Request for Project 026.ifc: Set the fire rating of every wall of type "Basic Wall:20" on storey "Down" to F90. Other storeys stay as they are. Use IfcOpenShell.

First a look at what the model holds.

```python
import ifcopenshell
import ifcopenshell.util.element

model = ifcopenshell.open("Project 026.ifc")
print(model.schema)
storey = next(s for s in model.by_type("IfcBuildingStorey") if s.Name == "Down")
walls = [e for e in ifcopenshell.util.element.get_decomposition(storey) if e.is_a("IfcWall")]
seen = {}
for e in walls:
    element_type = ifcopenshell.util.element.get_type(e)
    key = (element_type.Name if element_type != e and element_type else None, ifcopenshell.util.element.get_pset(e, "Pset_WallCommon", "FireRating"))
    seen[key] = seen.get(key, 0) + 1
for (name, value), count in sorted(seen.items(), key=str):
    print(count, "x", name, "|", value)
```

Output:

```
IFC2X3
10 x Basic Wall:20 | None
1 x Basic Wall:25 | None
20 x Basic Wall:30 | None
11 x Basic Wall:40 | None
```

```python
import ifcopenshell
import ifcopenshell.api.pset
import ifcopenshell.util.element

model = ifcopenshell.open("Project 026.ifc")

storey = next(s for s in model.by_type("IfcBuildingStorey") if s.Name == "Down")
walls = [e for e in ifcopenshell.util.element.get_decomposition(storey) if e.is_a("IfcWall")]

count = 0
for e in walls:
    element_type = ifcopenshell.util.element.get_type(e)
    if element_type in (None, e) or element_type.Name != "Basic Wall:20":
        continue
    # add_pset returns the element's existing set when there is one.
    pset = ifcopenshell.api.pset.add_pset(model, product=e, name="Pset_WallCommon")
    ifcopenshell.api.pset.edit_pset(model, pset=pset, properties={"FireRating": "F90"})
    count += 1

print(count, "walls updated")

model.write("Project 026_rev.ifc")
```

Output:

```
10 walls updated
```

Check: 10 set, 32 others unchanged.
